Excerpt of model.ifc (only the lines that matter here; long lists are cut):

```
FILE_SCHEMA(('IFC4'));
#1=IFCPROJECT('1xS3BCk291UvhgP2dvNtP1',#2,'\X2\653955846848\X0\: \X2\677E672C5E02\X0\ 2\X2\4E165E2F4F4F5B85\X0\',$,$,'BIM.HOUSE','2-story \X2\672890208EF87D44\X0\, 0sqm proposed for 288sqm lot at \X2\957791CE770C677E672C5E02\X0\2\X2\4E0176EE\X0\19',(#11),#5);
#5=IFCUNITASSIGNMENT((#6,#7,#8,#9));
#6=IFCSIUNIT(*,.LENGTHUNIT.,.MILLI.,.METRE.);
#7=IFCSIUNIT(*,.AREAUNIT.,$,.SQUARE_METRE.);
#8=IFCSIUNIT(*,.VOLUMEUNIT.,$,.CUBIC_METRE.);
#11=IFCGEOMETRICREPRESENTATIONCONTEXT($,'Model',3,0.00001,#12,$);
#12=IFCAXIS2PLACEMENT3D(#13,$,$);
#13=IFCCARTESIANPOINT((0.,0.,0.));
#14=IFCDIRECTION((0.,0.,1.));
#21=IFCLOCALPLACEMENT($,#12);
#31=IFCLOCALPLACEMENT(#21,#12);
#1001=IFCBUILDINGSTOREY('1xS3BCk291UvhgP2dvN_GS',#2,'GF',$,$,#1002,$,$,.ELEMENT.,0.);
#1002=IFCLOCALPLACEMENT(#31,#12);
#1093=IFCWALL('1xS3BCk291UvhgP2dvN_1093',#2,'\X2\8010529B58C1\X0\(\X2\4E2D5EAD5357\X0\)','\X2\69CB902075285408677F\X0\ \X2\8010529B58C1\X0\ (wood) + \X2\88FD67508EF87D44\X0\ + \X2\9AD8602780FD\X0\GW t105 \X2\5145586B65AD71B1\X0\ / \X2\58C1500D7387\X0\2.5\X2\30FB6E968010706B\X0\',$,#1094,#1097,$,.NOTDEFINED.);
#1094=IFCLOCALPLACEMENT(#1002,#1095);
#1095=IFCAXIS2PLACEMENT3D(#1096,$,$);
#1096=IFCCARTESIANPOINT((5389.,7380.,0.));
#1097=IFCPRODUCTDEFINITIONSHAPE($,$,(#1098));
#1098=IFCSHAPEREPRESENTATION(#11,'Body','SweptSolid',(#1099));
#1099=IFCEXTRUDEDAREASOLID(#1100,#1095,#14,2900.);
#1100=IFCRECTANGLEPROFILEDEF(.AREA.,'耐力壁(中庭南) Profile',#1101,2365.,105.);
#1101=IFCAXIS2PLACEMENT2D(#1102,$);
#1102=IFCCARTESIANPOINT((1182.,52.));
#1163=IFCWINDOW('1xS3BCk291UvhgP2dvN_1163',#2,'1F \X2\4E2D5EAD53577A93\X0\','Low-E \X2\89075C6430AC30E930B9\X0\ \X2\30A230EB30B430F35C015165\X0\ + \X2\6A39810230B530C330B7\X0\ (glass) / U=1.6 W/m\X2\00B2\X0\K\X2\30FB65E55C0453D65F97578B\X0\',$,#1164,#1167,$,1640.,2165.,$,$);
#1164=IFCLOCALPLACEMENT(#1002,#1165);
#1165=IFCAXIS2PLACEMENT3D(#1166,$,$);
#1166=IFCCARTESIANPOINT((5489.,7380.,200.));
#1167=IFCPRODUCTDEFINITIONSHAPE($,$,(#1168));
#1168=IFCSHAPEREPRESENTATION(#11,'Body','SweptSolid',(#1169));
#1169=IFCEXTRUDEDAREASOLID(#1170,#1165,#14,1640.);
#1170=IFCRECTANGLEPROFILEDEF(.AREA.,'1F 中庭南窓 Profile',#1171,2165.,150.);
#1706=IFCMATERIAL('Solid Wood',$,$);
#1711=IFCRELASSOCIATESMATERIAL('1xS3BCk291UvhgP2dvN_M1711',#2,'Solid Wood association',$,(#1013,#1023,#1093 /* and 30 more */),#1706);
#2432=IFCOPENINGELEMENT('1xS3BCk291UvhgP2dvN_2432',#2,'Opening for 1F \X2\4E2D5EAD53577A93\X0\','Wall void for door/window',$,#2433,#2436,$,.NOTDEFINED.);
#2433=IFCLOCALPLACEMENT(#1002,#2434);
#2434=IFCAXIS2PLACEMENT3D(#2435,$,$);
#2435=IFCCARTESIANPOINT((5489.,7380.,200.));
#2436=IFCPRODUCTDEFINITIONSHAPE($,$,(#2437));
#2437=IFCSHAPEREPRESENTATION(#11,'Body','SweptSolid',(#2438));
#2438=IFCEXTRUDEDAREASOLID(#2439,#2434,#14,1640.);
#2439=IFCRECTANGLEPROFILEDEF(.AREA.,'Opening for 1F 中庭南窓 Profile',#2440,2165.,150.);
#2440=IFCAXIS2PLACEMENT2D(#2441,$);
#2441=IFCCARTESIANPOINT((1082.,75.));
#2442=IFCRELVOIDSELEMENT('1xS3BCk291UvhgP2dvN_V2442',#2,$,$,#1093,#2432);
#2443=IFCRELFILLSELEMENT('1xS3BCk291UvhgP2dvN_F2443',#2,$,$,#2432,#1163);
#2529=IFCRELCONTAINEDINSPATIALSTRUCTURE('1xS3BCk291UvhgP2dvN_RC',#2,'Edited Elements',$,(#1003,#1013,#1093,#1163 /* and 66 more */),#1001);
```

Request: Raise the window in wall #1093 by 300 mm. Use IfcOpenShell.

```python
import numpy as np
import ifcopenshell
import ifcopenshell.api.geometry
import ifcopenshell.util.placement
import ifcopenshell.util.unit

model = ifcopenshell.open("model.ifc")
unit_scale = ifcopenshell.util.unit.calculate_unit_scale(model)

window = model.by_id(1163)
opening = window.FillsVoids[0].RelatingOpeningElement
dz = 0.3 / unit_scale

shift = np.array([0.0, 0.0, dz])
# The window is not placed relative to its opening, so move both.
for product in (opening, window):
    matrix = ifcopenshell.util.placement.get_local_placement(product.ObjectPlacement)
    matrix[:3, 3] += shift
    ifcopenshell.api.geometry.edit_object_placement(model, product=product, matrix=matrix, is_si=False)

print(f"moved by {dz * unit_scale:+.3f} m")

model.write("model_v2.ifc")
```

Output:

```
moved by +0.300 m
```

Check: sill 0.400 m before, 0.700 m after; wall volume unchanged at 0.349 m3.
